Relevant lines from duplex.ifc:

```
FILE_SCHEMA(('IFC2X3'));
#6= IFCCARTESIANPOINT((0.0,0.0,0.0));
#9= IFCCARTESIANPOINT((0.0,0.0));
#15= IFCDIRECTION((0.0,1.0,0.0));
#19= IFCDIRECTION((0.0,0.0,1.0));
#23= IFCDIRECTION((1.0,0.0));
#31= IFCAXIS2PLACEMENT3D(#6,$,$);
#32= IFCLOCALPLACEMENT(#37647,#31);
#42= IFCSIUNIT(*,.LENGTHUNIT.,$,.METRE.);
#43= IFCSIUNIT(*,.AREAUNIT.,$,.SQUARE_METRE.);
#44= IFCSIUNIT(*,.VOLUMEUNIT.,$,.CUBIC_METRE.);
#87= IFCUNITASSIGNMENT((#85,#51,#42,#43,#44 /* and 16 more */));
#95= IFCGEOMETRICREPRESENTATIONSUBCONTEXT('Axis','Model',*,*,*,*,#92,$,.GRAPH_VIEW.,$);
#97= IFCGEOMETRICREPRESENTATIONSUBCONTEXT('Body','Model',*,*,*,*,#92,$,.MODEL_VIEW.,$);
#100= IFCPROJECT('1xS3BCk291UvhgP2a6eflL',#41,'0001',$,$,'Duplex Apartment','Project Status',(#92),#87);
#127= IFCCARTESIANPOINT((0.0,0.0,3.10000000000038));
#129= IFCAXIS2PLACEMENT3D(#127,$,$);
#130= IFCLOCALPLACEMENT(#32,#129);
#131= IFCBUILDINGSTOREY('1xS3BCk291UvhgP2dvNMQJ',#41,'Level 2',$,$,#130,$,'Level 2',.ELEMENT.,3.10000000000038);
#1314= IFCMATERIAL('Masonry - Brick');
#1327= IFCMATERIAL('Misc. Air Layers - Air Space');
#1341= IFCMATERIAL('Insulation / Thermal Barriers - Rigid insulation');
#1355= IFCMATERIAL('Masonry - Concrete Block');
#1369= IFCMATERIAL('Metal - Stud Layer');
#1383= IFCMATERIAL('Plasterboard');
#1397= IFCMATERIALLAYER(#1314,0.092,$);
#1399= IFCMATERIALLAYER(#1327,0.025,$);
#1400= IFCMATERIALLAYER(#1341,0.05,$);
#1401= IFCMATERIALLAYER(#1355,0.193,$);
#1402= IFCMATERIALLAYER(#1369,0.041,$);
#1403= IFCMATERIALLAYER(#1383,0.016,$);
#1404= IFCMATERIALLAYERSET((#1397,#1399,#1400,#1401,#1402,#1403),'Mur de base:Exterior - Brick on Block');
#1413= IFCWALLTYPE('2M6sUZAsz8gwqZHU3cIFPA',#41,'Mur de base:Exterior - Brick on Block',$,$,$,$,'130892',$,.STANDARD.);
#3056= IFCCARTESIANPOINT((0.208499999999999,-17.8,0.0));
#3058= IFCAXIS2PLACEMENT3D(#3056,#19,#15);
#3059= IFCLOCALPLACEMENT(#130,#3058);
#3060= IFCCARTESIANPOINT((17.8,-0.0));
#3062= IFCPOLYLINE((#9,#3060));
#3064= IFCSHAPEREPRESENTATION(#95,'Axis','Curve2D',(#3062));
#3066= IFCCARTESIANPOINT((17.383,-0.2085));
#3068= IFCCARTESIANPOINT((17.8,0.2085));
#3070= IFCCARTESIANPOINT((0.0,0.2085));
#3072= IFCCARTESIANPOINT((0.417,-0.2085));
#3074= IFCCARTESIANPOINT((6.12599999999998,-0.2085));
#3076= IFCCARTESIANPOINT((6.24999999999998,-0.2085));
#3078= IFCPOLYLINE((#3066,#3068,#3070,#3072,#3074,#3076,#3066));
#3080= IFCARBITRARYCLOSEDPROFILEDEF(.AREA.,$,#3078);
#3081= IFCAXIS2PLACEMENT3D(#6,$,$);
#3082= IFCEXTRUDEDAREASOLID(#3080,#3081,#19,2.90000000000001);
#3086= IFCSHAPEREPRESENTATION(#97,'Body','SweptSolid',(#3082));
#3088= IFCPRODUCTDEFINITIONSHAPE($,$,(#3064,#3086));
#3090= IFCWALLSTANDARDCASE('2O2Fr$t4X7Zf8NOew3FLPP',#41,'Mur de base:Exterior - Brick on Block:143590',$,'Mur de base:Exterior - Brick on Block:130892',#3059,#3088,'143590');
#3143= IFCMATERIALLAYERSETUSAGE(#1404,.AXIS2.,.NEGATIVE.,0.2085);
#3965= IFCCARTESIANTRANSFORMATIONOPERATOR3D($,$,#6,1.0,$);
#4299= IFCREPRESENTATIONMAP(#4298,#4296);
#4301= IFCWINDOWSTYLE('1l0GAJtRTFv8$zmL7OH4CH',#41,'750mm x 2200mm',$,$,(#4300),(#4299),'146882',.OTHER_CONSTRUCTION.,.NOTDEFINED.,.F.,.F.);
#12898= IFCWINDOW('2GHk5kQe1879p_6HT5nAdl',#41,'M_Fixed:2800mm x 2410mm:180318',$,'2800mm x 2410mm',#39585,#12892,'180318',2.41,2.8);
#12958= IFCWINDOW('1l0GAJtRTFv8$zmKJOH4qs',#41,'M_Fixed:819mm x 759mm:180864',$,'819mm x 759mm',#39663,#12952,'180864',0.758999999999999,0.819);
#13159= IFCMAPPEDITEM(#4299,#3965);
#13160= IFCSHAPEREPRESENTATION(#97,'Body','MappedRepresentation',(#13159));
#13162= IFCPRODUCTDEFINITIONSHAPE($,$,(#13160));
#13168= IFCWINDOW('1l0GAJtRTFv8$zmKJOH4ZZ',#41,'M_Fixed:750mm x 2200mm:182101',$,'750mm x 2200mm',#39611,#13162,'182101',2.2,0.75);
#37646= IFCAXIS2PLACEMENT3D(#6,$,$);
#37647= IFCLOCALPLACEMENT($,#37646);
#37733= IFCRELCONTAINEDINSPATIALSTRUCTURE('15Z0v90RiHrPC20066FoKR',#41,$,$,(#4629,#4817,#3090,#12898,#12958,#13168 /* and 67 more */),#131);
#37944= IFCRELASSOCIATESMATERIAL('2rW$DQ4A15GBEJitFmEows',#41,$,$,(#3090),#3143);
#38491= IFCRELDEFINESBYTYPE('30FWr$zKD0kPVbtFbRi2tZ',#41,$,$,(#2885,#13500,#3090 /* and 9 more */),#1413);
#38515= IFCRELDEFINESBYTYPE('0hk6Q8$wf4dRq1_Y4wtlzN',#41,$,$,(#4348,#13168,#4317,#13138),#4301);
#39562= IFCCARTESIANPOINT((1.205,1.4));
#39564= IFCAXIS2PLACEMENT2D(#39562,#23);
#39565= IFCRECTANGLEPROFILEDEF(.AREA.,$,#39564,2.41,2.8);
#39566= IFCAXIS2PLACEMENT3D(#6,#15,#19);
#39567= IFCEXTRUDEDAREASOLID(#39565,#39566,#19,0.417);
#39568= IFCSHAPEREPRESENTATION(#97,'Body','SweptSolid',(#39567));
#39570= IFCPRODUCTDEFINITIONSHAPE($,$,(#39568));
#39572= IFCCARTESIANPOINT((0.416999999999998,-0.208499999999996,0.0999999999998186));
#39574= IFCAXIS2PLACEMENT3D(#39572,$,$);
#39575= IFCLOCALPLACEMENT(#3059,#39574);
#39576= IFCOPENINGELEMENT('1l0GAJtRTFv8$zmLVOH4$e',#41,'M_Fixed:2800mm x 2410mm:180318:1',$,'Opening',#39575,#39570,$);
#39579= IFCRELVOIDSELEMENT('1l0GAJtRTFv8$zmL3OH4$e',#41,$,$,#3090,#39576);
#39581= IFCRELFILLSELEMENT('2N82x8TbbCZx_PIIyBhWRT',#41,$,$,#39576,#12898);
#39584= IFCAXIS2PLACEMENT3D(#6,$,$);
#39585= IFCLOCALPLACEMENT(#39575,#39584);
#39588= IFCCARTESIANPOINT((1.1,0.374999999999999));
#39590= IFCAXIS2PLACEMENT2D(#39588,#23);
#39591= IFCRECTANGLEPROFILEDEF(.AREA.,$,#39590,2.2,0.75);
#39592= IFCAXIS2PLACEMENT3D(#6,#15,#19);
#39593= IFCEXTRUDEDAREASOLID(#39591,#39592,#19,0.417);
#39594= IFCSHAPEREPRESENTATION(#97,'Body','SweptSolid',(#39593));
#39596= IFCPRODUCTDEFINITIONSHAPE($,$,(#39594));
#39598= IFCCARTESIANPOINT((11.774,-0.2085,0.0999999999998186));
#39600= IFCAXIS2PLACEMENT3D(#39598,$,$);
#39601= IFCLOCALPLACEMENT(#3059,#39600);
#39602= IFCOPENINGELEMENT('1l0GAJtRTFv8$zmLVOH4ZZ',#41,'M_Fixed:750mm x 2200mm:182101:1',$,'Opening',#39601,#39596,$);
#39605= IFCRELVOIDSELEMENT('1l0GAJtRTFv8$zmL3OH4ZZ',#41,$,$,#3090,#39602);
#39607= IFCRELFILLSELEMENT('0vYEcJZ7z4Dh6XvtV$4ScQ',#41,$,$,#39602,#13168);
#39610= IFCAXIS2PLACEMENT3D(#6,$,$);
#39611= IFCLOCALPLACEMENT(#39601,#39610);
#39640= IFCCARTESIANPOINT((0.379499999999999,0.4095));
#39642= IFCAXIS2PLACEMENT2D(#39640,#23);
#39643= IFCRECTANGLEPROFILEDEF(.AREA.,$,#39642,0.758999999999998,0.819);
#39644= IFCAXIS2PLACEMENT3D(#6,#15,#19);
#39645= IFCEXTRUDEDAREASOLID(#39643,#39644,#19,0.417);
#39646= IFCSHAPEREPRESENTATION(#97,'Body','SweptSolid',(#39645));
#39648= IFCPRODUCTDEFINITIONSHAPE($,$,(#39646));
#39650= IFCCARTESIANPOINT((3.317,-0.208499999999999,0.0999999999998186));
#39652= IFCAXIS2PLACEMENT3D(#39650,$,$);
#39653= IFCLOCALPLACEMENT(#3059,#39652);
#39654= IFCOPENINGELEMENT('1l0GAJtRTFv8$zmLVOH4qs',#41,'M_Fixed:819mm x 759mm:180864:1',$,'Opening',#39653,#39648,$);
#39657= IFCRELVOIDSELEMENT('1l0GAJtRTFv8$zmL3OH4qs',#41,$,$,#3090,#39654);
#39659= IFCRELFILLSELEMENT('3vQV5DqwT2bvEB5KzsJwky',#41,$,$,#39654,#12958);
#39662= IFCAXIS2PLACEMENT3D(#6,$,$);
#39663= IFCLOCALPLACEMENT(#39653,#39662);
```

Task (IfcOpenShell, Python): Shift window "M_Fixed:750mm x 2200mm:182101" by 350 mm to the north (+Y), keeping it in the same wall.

```python
import ifcopenshell
import ifcopenshell.api.geometry
import ifcopenshell.util.placement
import ifcopenshell.util.unit

model = ifcopenshell.open("duplex.ifc")
unit_scale = ifcopenshell.util.unit.calculate_unit_scale(model)

window = model.by_guid("1l0GAJtRTFv8$zmKJOH4ZZ")
opening = window.FillsVoids[0].RelatingOpeningElement
wall = opening.VoidsElements[0].RelatingBuildingElement

wall_matrix = ifcopenshell.util.placement.get_local_placement(wall.ObjectPlacement)
shift = wall_matrix[:3, 0] * 0.35 / unit_scale
before = ifcopenshell.util.placement.get_local_placement(window.ObjectPlacement)[:3, 3].copy()

# The window is placed relative to its opening, so it follows when the opening moves.
matrix = ifcopenshell.util.placement.get_local_placement(opening.ObjectPlacement)
matrix[:3, 3] += shift
ifcopenshell.api.geometry.edit_object_placement(
    model, product=opening, matrix=matrix, is_si=False, should_transform_children=True
)

after = ifcopenshell.util.placement.get_local_placement(window.ObjectPlacement)[:3, 3]
print("window moved by", (after - before).round(3) + 0.0)

model.write("duplex_updated.ifc")
```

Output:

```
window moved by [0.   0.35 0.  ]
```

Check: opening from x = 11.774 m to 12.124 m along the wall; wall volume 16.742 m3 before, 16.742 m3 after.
